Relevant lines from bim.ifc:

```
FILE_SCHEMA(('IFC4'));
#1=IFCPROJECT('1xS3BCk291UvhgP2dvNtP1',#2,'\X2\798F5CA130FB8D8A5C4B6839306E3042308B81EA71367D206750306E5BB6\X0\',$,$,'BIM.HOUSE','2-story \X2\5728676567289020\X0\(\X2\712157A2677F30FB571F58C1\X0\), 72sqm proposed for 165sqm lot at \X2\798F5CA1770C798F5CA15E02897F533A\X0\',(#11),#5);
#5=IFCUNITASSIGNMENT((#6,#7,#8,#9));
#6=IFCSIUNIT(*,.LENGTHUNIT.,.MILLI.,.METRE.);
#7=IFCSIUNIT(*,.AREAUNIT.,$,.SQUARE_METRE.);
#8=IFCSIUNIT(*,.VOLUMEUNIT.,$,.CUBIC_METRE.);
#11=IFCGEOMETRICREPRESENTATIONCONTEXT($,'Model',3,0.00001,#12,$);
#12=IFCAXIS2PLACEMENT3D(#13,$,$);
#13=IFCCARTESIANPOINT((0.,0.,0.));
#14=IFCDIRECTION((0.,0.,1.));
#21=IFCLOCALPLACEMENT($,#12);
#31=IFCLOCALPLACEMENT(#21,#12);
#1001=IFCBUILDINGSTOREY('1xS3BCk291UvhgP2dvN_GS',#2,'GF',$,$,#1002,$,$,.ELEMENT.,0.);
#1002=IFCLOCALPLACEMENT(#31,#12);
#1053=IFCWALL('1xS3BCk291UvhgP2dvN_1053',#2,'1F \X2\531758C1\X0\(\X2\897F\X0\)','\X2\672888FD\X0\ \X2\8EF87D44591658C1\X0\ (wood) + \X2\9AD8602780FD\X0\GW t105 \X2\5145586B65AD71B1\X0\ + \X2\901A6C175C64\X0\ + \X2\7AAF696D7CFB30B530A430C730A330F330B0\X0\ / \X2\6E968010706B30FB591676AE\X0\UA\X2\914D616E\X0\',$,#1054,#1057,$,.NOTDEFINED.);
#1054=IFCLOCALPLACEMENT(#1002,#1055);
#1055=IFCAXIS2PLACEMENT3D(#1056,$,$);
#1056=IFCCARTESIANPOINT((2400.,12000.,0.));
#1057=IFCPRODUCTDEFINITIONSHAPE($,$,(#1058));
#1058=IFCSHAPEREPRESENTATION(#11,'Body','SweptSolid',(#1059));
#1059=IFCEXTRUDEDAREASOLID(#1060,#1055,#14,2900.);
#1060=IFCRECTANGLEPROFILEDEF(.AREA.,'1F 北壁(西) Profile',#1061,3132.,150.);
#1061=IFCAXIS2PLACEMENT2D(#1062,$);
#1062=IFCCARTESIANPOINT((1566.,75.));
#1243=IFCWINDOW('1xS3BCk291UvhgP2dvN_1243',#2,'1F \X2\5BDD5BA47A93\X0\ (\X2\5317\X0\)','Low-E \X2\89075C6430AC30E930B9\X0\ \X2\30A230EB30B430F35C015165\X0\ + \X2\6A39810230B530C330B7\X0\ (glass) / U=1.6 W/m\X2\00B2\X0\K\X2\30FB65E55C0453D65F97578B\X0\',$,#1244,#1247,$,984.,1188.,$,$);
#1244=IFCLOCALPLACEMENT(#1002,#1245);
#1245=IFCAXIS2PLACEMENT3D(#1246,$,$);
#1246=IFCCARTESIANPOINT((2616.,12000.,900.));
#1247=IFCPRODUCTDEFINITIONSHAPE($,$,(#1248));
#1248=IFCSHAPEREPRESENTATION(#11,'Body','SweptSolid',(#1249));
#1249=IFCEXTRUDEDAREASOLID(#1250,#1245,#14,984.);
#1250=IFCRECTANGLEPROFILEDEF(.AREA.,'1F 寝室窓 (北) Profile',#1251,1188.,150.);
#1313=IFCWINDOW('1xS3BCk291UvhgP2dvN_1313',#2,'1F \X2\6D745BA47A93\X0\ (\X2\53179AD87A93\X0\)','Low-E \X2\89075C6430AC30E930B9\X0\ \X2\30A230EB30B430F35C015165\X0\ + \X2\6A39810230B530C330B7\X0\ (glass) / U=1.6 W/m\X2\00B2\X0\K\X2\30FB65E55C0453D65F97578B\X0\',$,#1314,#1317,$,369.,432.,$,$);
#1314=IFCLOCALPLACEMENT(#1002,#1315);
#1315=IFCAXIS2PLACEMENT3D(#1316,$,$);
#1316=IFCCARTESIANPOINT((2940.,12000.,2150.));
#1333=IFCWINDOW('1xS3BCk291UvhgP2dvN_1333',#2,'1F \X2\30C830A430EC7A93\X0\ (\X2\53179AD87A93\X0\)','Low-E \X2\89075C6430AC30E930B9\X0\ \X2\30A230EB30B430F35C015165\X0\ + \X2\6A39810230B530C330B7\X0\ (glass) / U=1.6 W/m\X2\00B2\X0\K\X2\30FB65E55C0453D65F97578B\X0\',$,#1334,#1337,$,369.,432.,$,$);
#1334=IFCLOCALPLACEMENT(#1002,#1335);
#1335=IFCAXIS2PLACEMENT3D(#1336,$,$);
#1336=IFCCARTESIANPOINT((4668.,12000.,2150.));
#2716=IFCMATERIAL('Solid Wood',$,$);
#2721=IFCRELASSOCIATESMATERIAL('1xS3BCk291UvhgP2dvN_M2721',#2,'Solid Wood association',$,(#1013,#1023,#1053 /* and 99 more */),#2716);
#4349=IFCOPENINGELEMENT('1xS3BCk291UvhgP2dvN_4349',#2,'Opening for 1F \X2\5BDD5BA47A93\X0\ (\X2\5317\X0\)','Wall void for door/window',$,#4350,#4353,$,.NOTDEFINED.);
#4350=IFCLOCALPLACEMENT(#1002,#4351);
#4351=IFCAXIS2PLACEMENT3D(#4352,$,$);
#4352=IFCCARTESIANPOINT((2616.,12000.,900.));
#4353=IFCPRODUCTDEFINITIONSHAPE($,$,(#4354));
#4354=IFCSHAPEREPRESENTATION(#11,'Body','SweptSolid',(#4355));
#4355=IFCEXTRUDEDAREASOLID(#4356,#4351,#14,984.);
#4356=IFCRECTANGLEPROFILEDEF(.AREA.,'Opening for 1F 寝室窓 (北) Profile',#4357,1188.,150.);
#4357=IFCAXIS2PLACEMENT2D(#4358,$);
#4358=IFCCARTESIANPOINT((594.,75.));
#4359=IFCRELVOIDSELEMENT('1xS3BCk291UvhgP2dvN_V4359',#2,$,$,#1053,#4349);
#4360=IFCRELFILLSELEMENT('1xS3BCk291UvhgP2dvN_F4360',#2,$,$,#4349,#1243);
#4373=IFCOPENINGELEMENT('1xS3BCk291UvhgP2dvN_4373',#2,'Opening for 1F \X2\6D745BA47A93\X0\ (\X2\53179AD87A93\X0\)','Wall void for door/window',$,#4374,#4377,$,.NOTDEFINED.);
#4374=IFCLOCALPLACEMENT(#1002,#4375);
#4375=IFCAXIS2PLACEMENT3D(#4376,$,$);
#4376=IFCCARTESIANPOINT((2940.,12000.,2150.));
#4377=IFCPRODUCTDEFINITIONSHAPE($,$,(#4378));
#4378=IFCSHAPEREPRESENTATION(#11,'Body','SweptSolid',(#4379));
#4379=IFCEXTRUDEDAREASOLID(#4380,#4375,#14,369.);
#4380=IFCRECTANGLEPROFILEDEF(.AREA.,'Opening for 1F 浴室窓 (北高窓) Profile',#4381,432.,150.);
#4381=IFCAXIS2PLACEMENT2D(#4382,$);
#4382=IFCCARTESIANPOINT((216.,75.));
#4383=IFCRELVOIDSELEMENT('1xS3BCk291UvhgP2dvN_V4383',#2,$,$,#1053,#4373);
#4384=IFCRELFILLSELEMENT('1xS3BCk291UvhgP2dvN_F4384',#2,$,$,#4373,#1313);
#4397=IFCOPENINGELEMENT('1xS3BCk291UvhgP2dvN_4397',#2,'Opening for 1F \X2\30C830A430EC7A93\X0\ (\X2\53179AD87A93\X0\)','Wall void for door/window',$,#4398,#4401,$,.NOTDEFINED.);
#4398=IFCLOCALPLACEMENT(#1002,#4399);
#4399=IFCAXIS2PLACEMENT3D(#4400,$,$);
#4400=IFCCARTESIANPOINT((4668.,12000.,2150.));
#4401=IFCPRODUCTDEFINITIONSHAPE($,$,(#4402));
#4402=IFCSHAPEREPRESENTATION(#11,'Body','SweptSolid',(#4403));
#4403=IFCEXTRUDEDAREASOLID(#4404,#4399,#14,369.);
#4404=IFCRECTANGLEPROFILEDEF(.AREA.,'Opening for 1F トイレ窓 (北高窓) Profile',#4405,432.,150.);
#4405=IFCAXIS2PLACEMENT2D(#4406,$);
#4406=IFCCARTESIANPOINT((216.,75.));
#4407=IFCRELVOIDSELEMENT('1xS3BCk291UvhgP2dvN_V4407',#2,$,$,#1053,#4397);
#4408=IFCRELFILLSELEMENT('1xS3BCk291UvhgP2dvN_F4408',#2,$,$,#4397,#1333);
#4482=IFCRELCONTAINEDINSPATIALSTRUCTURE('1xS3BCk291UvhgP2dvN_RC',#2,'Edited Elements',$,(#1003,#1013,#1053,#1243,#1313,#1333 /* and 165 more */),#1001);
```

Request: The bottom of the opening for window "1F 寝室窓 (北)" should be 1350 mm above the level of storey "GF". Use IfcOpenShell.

```python
import numpy as np
import ifcopenshell
import ifcopenshell.api.geometry
import ifcopenshell.geom
import ifcopenshell.util.element
import ifcopenshell.util.placement
import ifcopenshell.util.shape
import ifcopenshell.util.unit

model = ifcopenshell.open("bim.ifc")
unit_scale = ifcopenshell.util.unit.calculate_unit_scale(model)

window = model.by_guid("1xS3BCk291UvhgP2dvN_1243")
opening = window.FillsVoids[0].RelatingOpeningElement
storey = ifcopenshell.util.element.get_container(window, ifc_class="IfcBuildingStorey")
level = ifcopenshell.util.placement.get_local_placement(storey.ObjectPlacement)[2, 3]

# The opening's origin need not be at the sill, so measure its lowest point.
shape = ifcopenshell.geom.create_shape(ifcopenshell.geom.settings(), opening)
bottom = ifcopenshell.util.shape.get_shape_bottom_elevation(shape, shape.geometry) / unit_scale
dz = level + 1.35 / unit_scale - bottom

shift = np.array([0.0, 0.0, dz])
# The window is not placed relative to its opening, so move both.
for product in (opening, window):
    matrix = ifcopenshell.util.placement.get_local_placement(product.ObjectPlacement)
    matrix[:3, 3] += shift
    ifcopenshell.api.geometry.edit_object_placement(model, product=product, matrix=matrix, is_si=False)

print(f"moved by {dz * unit_scale:+.3f} m")

model.write("bim_v2.ifc")
```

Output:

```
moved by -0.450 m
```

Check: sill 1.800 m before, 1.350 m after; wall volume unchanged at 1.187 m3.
